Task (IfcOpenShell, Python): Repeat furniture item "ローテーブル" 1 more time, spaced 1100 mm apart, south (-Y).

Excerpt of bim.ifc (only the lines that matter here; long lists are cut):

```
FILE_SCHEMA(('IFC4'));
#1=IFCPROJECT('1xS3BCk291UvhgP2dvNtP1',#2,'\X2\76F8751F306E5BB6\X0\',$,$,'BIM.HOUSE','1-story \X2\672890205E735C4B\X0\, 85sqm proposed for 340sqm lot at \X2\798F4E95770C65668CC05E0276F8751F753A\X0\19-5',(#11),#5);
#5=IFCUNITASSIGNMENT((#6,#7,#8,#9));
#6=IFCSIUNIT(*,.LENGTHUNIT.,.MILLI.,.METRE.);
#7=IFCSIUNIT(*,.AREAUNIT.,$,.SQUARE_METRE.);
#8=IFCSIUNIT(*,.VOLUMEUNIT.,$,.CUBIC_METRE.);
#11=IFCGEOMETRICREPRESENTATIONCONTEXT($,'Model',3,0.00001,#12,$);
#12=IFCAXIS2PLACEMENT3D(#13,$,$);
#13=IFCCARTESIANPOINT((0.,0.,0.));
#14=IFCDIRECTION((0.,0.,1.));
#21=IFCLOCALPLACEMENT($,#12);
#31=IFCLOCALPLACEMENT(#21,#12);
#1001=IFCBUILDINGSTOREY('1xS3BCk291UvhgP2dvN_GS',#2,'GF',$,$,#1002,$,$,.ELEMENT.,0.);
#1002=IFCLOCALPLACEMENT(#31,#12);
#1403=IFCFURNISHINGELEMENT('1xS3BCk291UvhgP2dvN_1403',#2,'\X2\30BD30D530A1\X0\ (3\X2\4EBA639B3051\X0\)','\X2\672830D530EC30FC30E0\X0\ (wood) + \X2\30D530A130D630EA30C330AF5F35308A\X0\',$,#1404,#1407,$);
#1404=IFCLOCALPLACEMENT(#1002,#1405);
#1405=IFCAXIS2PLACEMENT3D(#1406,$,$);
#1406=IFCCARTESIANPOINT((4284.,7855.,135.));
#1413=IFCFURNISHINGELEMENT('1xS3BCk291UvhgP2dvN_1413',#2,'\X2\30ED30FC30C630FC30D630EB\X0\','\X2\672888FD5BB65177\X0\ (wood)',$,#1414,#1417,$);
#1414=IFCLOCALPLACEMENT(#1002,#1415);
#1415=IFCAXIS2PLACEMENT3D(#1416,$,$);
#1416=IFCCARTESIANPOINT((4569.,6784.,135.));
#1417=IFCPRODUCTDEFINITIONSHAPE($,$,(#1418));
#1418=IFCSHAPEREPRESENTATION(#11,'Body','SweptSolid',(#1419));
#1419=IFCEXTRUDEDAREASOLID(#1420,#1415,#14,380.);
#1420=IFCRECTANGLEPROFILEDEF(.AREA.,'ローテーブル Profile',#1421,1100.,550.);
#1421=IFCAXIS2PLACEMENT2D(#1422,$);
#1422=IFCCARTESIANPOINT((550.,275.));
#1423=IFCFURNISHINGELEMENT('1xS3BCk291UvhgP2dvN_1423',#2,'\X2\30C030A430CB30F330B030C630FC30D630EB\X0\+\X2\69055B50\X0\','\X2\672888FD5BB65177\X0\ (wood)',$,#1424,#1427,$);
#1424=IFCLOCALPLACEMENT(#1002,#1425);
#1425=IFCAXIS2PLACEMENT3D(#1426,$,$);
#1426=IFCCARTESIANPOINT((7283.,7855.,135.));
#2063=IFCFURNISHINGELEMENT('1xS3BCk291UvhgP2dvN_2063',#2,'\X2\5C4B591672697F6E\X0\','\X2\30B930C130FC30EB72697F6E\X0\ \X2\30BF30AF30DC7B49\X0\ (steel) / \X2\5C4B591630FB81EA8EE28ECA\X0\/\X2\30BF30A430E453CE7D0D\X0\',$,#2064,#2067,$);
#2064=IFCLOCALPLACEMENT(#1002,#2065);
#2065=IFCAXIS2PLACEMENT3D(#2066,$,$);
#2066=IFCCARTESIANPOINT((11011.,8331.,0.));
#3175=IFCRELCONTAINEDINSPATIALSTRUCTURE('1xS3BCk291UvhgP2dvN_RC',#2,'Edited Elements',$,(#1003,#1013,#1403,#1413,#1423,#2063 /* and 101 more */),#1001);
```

```python
import numpy as np
import ifcopenshell
import ifcopenshell.api.geometry
import ifcopenshell.api.root
import ifcopenshell.util.element
import ifcopenshell.util.placement
import ifcopenshell.util.unit

model = ifcopenshell.open("bim.ifc")
unit_scale = ifcopenshell.util.unit.calculate_unit_scale(model)


def reuse_history(source, copy):
    """copy_class also copies each property set's owner history, people and application; keep the originals."""
    for rel in copy.IsDefinedBy:
        if rel.is_a("IfcRelDefinesByProperties") and (history := rel.RelatingPropertyDefinition.OwnerHistory):
            rel.RelatingPropertyDefinition.OwnerHistory = source.OwnerHistory
            ifcopenshell.util.element.remove_deep2(model, history)


source = model.by_guid("1xS3BCk291UvhgP2dvN_1413")
base = ifcopenshell.util.placement.get_local_placement(source.ObjectPlacement)
step = np.array([0.0, -1.0, 0.0]) * 1.1 / unit_scale

for i in range(1, 2):
    copy = ifcopenshell.api.root.copy_class(model, product=source)
    copy.Representation = ifcopenshell.util.element.copy_deep(
        model, source.Representation, exclude=["IfcGeometricRepresentationContext", "IfcRepresentationMap"]
    )
    reuse_history(source, copy)
    matrix = base.copy()
    matrix[:3, 3] += i * step
    print("added at", matrix[:3, 3].round(3) + 0.0)
    ifcopenshell.api.geometry.edit_object_placement(model, product=copy, matrix=matrix, is_si=False)

model.write("bim_v2.ifc")
```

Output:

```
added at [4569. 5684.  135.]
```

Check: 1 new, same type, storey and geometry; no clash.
